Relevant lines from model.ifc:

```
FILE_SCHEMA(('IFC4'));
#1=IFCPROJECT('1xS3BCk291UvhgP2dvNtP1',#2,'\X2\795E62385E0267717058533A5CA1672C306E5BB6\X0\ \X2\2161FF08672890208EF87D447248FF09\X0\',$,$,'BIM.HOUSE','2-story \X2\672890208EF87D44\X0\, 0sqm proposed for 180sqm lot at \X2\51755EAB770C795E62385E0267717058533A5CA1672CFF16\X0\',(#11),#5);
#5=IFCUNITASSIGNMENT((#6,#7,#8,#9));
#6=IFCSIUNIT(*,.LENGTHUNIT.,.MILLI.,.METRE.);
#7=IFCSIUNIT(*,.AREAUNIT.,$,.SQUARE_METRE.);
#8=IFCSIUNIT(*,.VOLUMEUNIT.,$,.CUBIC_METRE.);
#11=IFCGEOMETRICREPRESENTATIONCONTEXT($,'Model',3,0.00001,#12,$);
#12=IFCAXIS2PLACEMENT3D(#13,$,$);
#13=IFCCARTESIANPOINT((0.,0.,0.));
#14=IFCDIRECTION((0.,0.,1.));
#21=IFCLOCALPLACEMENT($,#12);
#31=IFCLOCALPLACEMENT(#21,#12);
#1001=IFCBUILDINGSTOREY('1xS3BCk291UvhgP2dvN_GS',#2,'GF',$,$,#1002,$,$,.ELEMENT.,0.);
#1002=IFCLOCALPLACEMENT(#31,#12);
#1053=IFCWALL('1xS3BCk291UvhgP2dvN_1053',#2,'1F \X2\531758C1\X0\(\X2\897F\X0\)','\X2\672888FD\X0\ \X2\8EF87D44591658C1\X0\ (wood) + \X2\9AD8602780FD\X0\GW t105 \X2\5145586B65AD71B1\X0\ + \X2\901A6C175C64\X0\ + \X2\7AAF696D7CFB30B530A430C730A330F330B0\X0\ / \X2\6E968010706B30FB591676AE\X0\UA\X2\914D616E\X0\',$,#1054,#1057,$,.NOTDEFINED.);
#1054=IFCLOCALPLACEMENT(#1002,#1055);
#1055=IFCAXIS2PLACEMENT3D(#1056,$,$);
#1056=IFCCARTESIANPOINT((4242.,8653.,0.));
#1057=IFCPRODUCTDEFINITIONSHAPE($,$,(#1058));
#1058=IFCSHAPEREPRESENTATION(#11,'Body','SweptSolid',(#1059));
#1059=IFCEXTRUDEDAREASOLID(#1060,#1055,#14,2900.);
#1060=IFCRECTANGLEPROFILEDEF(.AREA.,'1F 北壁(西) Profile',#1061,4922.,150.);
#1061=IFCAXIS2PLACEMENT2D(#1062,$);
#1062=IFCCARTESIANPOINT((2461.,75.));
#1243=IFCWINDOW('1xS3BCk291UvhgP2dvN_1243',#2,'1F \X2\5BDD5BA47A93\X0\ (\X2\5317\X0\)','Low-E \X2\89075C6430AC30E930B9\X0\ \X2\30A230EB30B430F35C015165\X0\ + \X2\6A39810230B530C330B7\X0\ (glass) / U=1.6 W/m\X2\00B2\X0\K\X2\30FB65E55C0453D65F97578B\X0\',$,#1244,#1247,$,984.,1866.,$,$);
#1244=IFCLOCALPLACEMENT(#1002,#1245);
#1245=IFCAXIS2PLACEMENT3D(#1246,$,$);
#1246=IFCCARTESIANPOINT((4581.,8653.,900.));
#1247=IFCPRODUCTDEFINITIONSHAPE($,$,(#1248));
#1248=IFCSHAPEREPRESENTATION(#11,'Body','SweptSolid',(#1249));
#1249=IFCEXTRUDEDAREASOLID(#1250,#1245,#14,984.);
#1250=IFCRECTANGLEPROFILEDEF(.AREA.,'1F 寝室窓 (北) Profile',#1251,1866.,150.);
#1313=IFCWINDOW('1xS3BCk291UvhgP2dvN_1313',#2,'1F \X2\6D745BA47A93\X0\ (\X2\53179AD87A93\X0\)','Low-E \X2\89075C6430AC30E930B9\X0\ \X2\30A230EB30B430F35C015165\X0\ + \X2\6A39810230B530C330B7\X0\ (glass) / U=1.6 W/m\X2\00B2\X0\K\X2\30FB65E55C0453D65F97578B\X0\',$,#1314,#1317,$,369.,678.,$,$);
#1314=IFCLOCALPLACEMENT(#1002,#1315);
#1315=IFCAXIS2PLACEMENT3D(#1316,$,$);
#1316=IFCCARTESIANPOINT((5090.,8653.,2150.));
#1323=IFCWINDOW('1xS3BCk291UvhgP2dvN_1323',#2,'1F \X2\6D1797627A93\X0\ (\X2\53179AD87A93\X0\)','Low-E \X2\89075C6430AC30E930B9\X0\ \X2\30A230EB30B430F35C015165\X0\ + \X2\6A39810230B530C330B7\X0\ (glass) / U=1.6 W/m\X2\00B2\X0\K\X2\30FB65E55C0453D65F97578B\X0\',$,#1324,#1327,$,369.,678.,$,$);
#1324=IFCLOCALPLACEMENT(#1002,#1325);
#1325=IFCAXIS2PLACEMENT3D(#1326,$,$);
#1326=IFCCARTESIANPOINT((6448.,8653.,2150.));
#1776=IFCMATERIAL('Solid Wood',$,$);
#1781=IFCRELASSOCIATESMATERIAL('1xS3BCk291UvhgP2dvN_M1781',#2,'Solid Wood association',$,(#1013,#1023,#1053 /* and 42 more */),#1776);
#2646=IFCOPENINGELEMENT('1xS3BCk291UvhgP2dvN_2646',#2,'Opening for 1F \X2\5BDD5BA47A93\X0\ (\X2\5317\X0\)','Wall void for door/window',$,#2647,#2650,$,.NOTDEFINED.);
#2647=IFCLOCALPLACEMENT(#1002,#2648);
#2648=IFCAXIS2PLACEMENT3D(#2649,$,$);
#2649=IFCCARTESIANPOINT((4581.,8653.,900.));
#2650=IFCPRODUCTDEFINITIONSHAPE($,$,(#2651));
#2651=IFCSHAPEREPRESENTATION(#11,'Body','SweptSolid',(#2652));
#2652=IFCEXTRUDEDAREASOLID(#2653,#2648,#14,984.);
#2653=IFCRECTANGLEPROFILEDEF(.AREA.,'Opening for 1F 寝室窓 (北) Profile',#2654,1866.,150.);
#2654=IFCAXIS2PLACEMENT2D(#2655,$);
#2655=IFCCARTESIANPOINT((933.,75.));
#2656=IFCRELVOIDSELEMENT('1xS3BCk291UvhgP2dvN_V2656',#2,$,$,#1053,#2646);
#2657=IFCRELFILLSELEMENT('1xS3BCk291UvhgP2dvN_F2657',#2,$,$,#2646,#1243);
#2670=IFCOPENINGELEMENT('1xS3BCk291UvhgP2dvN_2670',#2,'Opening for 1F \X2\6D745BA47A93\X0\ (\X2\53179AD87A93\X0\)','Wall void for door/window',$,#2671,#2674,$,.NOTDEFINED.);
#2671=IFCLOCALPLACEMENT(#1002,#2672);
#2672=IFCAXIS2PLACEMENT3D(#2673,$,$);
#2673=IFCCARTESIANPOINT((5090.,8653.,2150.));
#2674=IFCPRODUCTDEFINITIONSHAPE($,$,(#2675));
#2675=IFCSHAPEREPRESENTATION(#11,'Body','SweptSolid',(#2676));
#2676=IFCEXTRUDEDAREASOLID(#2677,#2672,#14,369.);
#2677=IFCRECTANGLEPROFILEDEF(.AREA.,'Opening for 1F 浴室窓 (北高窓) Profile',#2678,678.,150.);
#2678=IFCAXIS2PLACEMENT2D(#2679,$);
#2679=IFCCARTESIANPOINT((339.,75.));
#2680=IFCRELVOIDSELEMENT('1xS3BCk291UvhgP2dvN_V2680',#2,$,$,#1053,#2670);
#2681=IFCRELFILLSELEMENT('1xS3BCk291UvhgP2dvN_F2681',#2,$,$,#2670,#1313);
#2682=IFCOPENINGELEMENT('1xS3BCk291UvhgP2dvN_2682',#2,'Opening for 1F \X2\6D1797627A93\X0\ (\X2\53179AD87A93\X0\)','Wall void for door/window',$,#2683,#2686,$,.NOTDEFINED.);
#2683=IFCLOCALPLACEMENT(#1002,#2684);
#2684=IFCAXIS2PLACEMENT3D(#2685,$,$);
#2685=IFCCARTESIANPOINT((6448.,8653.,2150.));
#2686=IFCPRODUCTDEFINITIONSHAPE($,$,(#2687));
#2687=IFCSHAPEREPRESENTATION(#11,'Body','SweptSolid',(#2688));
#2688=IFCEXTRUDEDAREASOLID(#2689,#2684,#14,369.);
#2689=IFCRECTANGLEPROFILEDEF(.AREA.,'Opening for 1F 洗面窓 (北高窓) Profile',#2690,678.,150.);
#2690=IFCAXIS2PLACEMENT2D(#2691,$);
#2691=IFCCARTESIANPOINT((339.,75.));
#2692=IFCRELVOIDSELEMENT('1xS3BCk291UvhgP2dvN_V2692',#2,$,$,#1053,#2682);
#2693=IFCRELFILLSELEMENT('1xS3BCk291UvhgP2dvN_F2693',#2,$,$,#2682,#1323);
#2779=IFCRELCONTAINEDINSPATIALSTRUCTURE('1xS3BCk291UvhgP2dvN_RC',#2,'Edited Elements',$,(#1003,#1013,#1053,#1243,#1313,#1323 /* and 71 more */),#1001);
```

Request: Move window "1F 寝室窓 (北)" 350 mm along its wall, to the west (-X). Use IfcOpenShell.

```python
import ifcopenshell
import ifcopenshell.api.geometry
import ifcopenshell.util.placement
import ifcopenshell.util.unit

model = ifcopenshell.open("model.ifc")
unit_scale = ifcopenshell.util.unit.calculate_unit_scale(model)

window = model.by_guid("1xS3BCk291UvhgP2dvN_1243")
opening = window.FillsVoids[0].RelatingOpeningElement
wall = opening.VoidsElements[0].RelatingBuildingElement

wall_matrix = ifcopenshell.util.placement.get_local_placement(wall.ObjectPlacement)
shift = wall_matrix[:3, 0] * -0.35 / unit_scale
before = ifcopenshell.util.placement.get_local_placement(window.ObjectPlacement)[:3, 3].copy()

# The window is not placed relative to its opening, so move both.
for product in (opening, window):
    matrix = ifcopenshell.util.placement.get_local_placement(product.ObjectPlacement)
    matrix[:3, 3] += shift
    ifcopenshell.api.geometry.edit_object_placement(model, product=product, matrix=matrix, is_si=False)

after = ifcopenshell.util.placement.get_local_placement(window.ObjectPlacement)[:3, 3]
print("window moved by", (after - before).round(3) + 0.0)

model.write("model_updated.ifc")
```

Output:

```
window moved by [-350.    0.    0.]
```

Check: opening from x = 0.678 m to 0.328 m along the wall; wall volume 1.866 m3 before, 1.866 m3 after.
